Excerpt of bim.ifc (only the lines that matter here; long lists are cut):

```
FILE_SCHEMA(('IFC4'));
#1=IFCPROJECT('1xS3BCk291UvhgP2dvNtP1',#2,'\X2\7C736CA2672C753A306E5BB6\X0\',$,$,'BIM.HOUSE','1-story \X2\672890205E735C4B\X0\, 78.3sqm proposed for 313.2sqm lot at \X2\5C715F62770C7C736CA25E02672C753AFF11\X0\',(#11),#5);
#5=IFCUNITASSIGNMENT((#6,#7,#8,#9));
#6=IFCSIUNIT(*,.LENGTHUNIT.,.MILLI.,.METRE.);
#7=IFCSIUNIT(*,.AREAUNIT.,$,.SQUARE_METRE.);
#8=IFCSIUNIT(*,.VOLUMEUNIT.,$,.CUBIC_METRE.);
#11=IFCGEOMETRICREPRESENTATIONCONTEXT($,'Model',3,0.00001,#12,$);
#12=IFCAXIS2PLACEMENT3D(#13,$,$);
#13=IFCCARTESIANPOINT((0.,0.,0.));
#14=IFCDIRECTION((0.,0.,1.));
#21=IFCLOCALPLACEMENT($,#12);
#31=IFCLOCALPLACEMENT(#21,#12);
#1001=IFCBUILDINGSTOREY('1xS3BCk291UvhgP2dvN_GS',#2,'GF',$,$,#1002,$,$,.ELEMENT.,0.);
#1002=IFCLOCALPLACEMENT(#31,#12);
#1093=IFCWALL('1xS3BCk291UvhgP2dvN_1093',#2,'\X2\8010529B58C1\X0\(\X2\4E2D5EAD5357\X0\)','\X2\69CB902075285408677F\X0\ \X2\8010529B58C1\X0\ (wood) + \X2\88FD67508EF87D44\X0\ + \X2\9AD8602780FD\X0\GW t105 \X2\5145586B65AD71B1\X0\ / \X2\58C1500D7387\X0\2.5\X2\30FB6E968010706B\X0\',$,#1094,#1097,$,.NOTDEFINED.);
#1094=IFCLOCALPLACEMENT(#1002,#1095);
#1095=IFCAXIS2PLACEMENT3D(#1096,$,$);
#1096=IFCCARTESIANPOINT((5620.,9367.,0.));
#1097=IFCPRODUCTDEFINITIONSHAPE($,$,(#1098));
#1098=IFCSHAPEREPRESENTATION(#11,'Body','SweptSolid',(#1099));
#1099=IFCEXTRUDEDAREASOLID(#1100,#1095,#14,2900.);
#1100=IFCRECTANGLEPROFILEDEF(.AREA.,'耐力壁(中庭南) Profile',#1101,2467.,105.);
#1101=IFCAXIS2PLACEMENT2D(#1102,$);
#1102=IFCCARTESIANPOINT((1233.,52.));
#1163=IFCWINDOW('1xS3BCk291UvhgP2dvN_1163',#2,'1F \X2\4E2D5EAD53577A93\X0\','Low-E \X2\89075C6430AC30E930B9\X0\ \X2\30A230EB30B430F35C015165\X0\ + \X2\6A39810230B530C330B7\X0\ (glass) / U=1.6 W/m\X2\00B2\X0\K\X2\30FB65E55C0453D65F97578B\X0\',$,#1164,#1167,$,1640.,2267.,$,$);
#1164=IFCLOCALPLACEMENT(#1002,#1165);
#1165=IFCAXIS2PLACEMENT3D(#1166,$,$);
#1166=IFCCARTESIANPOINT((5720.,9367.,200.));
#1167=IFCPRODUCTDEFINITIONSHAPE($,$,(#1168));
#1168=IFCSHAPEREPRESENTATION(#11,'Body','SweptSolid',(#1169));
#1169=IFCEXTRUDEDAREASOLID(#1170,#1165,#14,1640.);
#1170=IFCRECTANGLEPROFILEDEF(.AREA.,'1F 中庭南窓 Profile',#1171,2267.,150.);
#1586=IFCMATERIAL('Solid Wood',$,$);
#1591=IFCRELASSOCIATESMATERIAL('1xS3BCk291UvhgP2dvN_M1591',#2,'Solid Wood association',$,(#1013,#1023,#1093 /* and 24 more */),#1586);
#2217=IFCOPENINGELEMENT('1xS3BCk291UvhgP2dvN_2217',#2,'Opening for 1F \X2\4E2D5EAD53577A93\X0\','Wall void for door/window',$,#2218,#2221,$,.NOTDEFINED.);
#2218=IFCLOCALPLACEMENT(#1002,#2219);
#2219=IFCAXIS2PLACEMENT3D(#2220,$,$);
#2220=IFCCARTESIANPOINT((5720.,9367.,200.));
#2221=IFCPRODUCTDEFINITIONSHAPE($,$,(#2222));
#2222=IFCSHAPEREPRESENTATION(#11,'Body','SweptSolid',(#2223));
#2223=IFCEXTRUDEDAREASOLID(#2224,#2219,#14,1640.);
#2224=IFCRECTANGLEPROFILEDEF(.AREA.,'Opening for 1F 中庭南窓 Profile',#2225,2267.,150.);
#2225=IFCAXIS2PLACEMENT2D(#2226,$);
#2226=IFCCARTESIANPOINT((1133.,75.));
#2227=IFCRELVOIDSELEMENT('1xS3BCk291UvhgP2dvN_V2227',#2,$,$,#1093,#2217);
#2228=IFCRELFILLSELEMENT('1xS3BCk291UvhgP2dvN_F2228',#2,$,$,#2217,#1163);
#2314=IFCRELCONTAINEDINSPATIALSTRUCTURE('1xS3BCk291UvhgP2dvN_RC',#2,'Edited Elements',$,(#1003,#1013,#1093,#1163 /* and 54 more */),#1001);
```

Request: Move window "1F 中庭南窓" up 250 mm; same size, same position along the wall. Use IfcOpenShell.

```python
import numpy as np
import ifcopenshell
import ifcopenshell.api.geometry
import ifcopenshell.util.placement
import ifcopenshell.util.unit

model = ifcopenshell.open("bim.ifc")
unit_scale = ifcopenshell.util.unit.calculate_unit_scale(model)

window = model.by_guid("1xS3BCk291UvhgP2dvN_1163")
opening = window.FillsVoids[0].RelatingOpeningElement
dz = 0.25 / unit_scale

shift = np.array([0.0, 0.0, dz])
# The window is not placed relative to its opening, so move both.
for product in (opening, window):
    matrix = ifcopenshell.util.placement.get_local_placement(product.ObjectPlacement)
    matrix[:3, 3] += shift
    ifcopenshell.api.geometry.edit_object_placement(model, product=product, matrix=matrix, is_si=False)

print(f"moved by {dz * unit_scale:+.3f} m")

model.write("bim_updated.ifc")
```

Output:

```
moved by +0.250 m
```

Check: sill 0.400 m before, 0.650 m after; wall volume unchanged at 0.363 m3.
